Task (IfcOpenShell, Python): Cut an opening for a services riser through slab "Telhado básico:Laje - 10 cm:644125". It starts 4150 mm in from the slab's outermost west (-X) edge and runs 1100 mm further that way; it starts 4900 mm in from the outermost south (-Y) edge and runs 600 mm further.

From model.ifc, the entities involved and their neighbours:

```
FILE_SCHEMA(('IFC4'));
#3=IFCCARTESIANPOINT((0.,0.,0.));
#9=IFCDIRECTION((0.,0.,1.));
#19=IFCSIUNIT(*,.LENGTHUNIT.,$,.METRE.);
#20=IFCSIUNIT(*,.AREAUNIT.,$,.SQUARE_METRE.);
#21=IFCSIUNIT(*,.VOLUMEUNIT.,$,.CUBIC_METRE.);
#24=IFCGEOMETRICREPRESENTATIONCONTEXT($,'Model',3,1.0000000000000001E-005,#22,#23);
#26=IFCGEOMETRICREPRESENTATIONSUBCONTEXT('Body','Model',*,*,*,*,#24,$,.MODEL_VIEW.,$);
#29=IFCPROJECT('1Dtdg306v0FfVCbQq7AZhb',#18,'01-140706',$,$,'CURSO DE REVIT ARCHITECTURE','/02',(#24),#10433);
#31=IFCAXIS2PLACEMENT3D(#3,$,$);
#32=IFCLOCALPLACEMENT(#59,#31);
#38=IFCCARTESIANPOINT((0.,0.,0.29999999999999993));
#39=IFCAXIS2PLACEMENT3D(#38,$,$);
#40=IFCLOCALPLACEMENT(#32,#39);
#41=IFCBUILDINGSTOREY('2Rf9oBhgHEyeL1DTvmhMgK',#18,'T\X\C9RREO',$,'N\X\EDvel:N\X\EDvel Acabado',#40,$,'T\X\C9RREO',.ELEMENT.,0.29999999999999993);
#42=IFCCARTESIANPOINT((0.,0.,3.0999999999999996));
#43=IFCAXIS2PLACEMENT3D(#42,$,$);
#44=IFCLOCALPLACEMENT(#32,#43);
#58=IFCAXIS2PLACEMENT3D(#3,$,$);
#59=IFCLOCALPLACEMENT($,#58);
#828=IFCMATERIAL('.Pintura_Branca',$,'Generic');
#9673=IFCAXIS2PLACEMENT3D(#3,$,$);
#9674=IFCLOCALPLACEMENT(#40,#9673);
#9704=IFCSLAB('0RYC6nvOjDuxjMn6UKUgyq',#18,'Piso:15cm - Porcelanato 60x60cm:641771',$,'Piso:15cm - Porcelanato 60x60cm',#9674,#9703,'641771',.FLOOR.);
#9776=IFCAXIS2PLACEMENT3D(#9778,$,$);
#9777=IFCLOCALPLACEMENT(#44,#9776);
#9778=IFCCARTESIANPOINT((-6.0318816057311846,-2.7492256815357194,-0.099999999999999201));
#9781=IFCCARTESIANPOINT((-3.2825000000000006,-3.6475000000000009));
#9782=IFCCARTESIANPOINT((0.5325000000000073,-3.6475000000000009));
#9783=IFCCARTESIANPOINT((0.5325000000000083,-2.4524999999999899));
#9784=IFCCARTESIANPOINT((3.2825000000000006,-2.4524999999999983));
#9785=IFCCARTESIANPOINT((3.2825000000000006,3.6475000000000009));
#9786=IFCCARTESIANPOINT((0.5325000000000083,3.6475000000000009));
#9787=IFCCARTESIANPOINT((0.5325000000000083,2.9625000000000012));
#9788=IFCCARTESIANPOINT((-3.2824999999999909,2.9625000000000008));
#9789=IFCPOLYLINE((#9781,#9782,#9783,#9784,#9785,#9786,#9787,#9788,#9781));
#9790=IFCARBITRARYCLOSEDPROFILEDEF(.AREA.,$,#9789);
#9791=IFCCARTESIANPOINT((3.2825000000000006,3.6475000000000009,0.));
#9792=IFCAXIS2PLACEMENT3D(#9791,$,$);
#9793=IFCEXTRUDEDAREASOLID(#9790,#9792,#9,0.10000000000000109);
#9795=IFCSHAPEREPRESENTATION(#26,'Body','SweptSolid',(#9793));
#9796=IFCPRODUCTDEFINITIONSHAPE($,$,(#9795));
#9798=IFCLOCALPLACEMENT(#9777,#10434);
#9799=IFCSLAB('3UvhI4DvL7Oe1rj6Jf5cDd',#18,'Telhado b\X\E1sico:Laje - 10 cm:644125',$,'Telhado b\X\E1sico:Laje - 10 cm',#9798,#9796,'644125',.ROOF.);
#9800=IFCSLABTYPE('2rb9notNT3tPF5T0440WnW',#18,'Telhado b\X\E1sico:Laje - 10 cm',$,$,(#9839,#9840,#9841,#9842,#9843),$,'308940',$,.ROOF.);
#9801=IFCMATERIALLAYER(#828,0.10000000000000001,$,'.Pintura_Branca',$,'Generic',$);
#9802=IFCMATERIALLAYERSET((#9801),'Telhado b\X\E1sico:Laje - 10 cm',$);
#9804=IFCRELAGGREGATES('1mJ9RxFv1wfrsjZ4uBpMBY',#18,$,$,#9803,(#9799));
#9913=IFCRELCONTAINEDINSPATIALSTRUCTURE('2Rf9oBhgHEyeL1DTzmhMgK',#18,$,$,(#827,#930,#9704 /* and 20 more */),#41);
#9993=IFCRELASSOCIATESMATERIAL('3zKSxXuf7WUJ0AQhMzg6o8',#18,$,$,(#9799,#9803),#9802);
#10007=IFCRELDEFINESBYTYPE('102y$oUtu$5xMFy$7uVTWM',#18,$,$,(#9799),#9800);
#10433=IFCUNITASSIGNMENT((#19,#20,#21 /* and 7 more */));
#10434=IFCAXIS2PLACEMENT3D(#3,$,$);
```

```python
import numpy as np
import ifcopenshell
import ifcopenshell.api.feature
import ifcopenshell.api.geometry
import ifcopenshell.api.root
import ifcopenshell.geom
import ifcopenshell.util.placement
import ifcopenshell.util.representation
import ifcopenshell.util.shape
import ifcopenshell.util.unit

model = ifcopenshell.open("model.ifc")
unit_scale = ifcopenshell.util.unit.calculate_unit_scale(model)
settings = ifcopenshell.geom.settings()


def volume(element):
    """Net volume in cubic metres, openings subtracted."""
    shape = ifcopenshell.geom.create_shape(settings, element)
    return ifcopenshell.util.shape.get_volume(shape.geometry)


slab = model.by_guid("3UvhI4DvL7Oe1rj6Jf5cDd")
before = volume(slab)

# Extent in the slab's own axes, in metres. The edges named are its -X and -Y sides.
slab_shape = ifcopenshell.geom.create_shape(settings, slab)
vertices = ifcopenshell.util.shape.get_vertices(slab_shape.geometry)
x_min, y_min, bottom = vertices.min(axis=0)
top = vertices[:, 2].max()

opening = ifcopenshell.api.root.create_entity(model, ifc_class="IfcOpeningElement", name="Services riser opening", predefined_type="OPENING")
context = ifcopenshell.util.representation.get_context(model, "Model", "Body", "MODEL_VIEW")
width, depth = 1.1, 0.6
outline = [(0.0, 0.0), (width, 0.0), (width, depth), (0.0, depth), (0.0, 0.0)]
# Overshoot both faces by 50 mm so the cut is clean.
shape = ifcopenshell.api.geometry.add_slab_representation(
    model, context=context, depth=top - bottom + 0.1, polyline=outline
)
ifcopenshell.api.geometry.assign_representation(model, product=opening, representation=shape)

matrix = ifcopenshell.util.placement.get_local_placement(slab.ObjectPlacement)
matrix[:, 3] = matrix @ np.append(np.array([x_min + 4.15, y_min + 4.9, bottom - 0.05]) / unit_scale, 1.0)
ifcopenshell.api.geometry.edit_object_placement(model, product=opening, matrix=matrix, is_si=False)
ifcopenshell.api.feature.add_feature(model, feature=opening, element=slab)

after = volume(slab)

print(f"slab volume {before:.3f} -> {after:.3f} m3")

model.write("model_v2.ifc")
```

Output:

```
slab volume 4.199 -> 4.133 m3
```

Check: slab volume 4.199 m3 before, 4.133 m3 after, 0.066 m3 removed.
